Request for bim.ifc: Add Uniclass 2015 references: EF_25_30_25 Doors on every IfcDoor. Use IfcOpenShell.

First a look at what the model holds.

```python
import ifcopenshell

model = ifcopenshell.open("bim.ifc")
print(model.schema)
print("classifications:", [c.Name for c in model.by_type("IfcClassification")])
for ifc_class in ("IfcDoor", "IfcRoof", "IfcStair", "IfcWall", "IfcWindow"):
    print(ifc_class, len(model.by_type(ifc_class)))
```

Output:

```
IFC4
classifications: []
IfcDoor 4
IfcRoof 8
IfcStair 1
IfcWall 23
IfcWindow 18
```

```python
import ifcopenshell
import ifcopenshell.api.classification

model = ifcopenshell.open("bim.ifc")

system = ifcopenshell.api.classification.add_classification(model, classification="Uniclass 2015")

codes = {
    "IfcDoor": ("EF_25_30_25", "Doors"),
}
for ifc_class, (code, name) in codes.items():
    products = model.by_type(ifc_class)
    ifcopenshell.api.classification.add_reference(
        model, products=products, classification=system, identification=code, name=name
    )
    print(code, len(products))

model.write("bim_v2.ifc")
```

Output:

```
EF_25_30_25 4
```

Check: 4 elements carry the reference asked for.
